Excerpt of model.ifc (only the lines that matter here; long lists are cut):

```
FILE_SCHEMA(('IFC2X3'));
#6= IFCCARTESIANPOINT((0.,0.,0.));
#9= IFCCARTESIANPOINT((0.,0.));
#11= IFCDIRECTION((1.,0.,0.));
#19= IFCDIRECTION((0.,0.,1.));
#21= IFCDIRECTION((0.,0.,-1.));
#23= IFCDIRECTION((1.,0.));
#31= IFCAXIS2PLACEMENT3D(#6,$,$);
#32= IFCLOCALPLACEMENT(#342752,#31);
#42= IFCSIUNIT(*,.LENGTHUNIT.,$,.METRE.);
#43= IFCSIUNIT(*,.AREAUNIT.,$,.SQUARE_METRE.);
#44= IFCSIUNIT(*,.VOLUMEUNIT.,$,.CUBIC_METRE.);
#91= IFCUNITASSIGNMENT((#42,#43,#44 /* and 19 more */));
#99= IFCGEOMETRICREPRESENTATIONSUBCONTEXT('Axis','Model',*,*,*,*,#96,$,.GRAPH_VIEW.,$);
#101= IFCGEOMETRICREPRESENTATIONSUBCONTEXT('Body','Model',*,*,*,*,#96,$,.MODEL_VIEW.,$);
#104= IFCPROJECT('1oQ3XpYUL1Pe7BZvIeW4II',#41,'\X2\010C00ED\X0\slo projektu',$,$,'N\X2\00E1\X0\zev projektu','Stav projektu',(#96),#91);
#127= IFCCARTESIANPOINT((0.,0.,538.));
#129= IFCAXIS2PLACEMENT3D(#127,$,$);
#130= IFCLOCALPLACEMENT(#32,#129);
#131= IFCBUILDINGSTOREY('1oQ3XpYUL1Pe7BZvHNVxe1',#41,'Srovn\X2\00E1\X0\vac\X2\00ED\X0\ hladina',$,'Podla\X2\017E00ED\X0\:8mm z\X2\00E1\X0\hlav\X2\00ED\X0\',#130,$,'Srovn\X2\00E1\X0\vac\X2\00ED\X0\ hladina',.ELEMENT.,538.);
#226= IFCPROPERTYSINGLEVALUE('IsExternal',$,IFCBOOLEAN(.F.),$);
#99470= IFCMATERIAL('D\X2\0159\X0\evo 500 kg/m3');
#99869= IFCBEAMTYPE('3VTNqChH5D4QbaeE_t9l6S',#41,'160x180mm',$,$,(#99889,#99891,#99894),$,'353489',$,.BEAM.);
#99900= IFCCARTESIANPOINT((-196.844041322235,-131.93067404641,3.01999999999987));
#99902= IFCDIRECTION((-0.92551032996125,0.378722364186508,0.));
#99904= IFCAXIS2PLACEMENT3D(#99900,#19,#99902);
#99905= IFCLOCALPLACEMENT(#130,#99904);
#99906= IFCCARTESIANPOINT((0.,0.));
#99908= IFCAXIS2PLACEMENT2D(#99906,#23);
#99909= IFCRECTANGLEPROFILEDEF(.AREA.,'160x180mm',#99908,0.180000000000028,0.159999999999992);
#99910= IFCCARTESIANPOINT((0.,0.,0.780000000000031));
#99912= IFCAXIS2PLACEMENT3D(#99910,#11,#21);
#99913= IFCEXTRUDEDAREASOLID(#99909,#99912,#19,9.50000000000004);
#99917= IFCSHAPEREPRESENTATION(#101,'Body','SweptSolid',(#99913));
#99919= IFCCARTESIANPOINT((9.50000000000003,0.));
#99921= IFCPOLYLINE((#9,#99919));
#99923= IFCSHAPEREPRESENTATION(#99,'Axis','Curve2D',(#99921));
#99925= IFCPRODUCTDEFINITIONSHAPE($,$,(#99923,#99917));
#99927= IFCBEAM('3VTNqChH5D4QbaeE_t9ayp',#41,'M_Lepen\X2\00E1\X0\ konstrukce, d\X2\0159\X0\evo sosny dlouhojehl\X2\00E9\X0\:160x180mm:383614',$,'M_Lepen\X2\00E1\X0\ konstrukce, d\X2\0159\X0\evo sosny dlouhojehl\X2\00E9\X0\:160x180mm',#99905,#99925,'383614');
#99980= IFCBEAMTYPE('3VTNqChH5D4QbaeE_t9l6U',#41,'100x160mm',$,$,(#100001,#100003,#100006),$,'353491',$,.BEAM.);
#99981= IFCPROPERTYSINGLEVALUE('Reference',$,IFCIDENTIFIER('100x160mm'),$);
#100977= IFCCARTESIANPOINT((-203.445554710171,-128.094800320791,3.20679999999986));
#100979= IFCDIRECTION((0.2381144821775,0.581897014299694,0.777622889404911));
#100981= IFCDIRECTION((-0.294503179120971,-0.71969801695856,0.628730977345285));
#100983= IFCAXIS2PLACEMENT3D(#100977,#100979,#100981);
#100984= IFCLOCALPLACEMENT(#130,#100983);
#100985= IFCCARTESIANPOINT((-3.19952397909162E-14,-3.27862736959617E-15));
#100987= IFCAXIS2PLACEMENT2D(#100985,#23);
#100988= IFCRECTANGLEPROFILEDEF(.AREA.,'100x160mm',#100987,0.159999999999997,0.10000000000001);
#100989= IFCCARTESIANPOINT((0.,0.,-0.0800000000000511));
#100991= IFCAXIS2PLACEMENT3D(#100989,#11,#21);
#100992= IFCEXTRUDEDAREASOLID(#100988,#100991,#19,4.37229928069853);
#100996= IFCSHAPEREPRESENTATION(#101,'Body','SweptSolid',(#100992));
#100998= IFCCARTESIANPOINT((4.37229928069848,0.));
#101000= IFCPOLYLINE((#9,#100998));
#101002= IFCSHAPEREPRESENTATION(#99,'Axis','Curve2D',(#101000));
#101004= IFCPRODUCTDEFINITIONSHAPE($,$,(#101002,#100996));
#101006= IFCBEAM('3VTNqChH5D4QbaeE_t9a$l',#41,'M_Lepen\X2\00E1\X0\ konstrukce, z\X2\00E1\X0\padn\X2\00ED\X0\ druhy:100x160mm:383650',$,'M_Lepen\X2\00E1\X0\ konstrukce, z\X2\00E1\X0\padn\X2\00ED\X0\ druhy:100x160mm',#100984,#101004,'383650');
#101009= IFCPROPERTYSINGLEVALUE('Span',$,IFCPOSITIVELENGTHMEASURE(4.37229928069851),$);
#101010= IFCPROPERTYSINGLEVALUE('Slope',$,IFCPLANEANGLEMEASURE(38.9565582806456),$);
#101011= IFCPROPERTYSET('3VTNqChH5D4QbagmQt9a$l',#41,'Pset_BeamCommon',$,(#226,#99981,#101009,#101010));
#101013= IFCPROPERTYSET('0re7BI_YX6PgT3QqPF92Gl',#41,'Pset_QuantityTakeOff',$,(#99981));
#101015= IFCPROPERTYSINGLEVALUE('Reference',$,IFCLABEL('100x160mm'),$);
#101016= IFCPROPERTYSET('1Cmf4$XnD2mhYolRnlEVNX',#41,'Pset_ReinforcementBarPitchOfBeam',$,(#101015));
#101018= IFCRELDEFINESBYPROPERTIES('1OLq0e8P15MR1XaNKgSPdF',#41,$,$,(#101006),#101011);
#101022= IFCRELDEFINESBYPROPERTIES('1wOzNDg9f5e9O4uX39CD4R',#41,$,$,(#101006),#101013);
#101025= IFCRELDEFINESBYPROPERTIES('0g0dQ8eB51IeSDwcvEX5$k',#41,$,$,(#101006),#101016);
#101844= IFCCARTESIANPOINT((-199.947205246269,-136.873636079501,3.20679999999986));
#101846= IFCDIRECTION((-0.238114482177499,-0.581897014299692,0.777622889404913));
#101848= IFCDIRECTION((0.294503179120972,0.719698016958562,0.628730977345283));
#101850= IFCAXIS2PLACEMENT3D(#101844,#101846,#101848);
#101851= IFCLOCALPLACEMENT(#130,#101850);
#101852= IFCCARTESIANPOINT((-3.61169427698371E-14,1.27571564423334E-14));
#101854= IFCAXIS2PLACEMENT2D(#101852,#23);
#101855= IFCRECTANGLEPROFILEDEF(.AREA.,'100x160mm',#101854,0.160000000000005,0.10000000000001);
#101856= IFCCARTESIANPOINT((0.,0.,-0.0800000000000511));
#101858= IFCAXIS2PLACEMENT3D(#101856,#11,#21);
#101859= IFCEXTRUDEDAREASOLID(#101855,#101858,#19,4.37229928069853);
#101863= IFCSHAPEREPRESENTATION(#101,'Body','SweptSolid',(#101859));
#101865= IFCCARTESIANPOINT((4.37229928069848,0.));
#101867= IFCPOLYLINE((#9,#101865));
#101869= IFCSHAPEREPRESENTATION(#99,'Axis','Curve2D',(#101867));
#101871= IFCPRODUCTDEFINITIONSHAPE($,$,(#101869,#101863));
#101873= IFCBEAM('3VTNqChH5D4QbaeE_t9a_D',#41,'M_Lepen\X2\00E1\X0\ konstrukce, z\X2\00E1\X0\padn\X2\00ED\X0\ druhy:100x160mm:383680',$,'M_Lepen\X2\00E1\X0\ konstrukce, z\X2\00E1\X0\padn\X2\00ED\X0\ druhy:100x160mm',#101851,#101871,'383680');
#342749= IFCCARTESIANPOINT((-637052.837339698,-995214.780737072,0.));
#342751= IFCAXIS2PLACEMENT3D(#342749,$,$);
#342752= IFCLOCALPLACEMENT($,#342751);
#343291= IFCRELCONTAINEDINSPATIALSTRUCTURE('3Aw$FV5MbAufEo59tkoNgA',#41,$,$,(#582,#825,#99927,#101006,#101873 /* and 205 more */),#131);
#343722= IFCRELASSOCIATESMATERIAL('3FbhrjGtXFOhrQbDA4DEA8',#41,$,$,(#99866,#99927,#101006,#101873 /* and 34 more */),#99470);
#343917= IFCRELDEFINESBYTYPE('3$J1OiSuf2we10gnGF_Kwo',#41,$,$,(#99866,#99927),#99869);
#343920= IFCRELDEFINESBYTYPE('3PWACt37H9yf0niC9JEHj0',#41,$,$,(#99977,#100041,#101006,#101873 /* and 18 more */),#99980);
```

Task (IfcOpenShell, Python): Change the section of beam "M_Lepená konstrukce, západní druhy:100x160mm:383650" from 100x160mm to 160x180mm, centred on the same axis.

```python
import ifcopenshell
import ifcopenshell.api.pset
import ifcopenshell.api.type
import ifcopenshell.util.element
import ifcopenshell.util.representation

model = ifcopenshell.open("model.ifc")

member = model.by_guid("3VTNqChH5D4QbaeE_t9a$l")
source = next(p for p in model.by_type("IfcRectangleProfileDef") if p.ProfileName == "160x180mm")

body = ifcopenshell.util.representation.get_representation(member, "Model", "Body")
solid = body.Items[0]
old_profile = solid.SweptArea

# Copy the section's sizes but keep this member's own profile position.
profile = ifcopenshell.util.element.copy(model, source)
profile.Position = old_profile.Position
solid.SweptArea = profile
if not model.get_total_inverses(old_profile):
    ifcopenshell.util.element.remove_deep2(model, old_profile)

new_type = model.by_guid("3VTNqChH5D4QbaeE_t9l6S")
ifcopenshell.api.type.assign_type(
    model, related_objects=[member], relating_type=new_type, should_map_representations=False
)
member.Name = member.Name.replace("100x160mm", "160x180mm")
member.ObjectType = "M_Lepená konstrukce, západní druhy:160x180mm"
pset = model.by_id(ifcopenshell.util.element.get_pset(member, "Pset_BeamCommon", should_inherit=False)["id"])
ifcopenshell.api.pset.edit_pset(model, pset=pset, properties={"Reference": "160x180mm"})
pset = model.by_id(ifcopenshell.util.element.get_pset(member, "Pset_QuantityTakeOff", should_inherit=False)["id"])
ifcopenshell.api.pset.edit_pset(model, pset=pset, properties={"Reference": "160x180mm"})
pset = model.by_id(ifcopenshell.util.element.get_pset(member, "Pset_ReinforcementBarPitchOfBeam", should_inherit=False)["id"])
ifcopenshell.api.pset.edit_pset(model, pset=pset, properties={"Reference": "160x180mm"})

print(solid.SweptArea)

model.write("model_v2.ifc")
```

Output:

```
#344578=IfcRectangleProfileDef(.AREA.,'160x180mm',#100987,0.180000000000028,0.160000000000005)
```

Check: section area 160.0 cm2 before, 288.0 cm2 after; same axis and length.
